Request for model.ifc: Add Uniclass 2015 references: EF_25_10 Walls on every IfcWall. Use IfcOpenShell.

First a look at what the model holds.

```python
import ifcopenshell

model = ifcopenshell.open("model.ifc")
print(model.schema)
print("classifications:", [c.Name for c in model.by_type("IfcClassification")])
for ifc_class in ("IfcDoor", "IfcRoof", "IfcStair", "IfcWall", "IfcWindow"):
    print(ifc_class, len(model.by_type(ifc_class)))
```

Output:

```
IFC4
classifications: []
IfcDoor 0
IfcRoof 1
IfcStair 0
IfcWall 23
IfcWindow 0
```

```python
import ifcopenshell
import ifcopenshell.api.classification

model = ifcopenshell.open("model.ifc")

system = ifcopenshell.api.classification.add_classification(model, classification="Uniclass 2015")

codes = {
    "IfcWall": ("EF_25_10", "Walls"),
}
for ifc_class, (code, name) in codes.items():
    products = model.by_type(ifc_class)
    ifcopenshell.api.classification.add_reference(
        model, products=products, classification=system, identification=code, name=name
    )
    print(code, len(products))

model.write("model_edited.ifc")
```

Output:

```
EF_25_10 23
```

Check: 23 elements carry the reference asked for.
